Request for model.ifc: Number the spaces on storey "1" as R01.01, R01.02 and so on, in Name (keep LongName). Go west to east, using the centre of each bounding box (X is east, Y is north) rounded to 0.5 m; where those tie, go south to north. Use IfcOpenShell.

First a look at what the model holds.

```python
import ifcopenshell
import ifcopenshell.util.element
import ifcopenshell.util.placement

model = ifcopenshell.open("model.ifc")
print(model.schema)
storey = next(s for s in model.by_type("IfcBuildingStorey") if s.Name == "1")
spaces = [e for e in ifcopenshell.util.element.get_decomposition(storey) if e.is_a("IfcSpace")]
for e in sorted(spaces, key=lambda e: e.id()):
    origin = ifcopenshell.util.placement.get_local_placement(e.ObjectPlacement)[:3, 3]
    print(e.id(), e.Name, e.LongName, origin.round(2) + 0.0, sep=" | ")
```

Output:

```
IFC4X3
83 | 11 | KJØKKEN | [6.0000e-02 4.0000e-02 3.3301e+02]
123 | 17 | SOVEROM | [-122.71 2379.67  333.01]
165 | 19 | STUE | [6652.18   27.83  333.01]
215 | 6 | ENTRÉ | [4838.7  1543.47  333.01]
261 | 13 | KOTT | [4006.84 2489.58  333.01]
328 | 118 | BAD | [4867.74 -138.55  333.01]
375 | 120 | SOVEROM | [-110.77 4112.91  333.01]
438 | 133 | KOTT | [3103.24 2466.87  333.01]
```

```python
import ifcopenshell
import ifcopenshell.geom
import ifcopenshell.util.element
import ifcopenshell.util.shape

model = ifcopenshell.open("model.ifc")
settings = ifcopenshell.geom.settings()
settings.set("use-world-coords", True)


def centre(element):
    shape = ifcopenshell.geom.create_shape(settings, element)
    return ifcopenshell.util.shape.get_bbox_centroid(shape.geometry)


storey = next(s for s in model.by_type("IfcBuildingStorey") if s.Name == "1")
spaces = [e for e in ifcopenshell.util.element.get_decomposition(storey) if e.is_a("IfcSpace")]

# Insertion points can sit at a corner or the storey origin, so sort by the geometry (in metres).
centres = {e: centre(e) for e in spaces}
spaces.sort(key=lambda e: (round(centres[e][0] / 0.5), centres[e][1]))

for i, e in enumerate(spaces, start=1):
    number = f"R01.{i:02d}"
    e.Name = number
    print(e.id(), number)

model.write("model_updated.ifc")
```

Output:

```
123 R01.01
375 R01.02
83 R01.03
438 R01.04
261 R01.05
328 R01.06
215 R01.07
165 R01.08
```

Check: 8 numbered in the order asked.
